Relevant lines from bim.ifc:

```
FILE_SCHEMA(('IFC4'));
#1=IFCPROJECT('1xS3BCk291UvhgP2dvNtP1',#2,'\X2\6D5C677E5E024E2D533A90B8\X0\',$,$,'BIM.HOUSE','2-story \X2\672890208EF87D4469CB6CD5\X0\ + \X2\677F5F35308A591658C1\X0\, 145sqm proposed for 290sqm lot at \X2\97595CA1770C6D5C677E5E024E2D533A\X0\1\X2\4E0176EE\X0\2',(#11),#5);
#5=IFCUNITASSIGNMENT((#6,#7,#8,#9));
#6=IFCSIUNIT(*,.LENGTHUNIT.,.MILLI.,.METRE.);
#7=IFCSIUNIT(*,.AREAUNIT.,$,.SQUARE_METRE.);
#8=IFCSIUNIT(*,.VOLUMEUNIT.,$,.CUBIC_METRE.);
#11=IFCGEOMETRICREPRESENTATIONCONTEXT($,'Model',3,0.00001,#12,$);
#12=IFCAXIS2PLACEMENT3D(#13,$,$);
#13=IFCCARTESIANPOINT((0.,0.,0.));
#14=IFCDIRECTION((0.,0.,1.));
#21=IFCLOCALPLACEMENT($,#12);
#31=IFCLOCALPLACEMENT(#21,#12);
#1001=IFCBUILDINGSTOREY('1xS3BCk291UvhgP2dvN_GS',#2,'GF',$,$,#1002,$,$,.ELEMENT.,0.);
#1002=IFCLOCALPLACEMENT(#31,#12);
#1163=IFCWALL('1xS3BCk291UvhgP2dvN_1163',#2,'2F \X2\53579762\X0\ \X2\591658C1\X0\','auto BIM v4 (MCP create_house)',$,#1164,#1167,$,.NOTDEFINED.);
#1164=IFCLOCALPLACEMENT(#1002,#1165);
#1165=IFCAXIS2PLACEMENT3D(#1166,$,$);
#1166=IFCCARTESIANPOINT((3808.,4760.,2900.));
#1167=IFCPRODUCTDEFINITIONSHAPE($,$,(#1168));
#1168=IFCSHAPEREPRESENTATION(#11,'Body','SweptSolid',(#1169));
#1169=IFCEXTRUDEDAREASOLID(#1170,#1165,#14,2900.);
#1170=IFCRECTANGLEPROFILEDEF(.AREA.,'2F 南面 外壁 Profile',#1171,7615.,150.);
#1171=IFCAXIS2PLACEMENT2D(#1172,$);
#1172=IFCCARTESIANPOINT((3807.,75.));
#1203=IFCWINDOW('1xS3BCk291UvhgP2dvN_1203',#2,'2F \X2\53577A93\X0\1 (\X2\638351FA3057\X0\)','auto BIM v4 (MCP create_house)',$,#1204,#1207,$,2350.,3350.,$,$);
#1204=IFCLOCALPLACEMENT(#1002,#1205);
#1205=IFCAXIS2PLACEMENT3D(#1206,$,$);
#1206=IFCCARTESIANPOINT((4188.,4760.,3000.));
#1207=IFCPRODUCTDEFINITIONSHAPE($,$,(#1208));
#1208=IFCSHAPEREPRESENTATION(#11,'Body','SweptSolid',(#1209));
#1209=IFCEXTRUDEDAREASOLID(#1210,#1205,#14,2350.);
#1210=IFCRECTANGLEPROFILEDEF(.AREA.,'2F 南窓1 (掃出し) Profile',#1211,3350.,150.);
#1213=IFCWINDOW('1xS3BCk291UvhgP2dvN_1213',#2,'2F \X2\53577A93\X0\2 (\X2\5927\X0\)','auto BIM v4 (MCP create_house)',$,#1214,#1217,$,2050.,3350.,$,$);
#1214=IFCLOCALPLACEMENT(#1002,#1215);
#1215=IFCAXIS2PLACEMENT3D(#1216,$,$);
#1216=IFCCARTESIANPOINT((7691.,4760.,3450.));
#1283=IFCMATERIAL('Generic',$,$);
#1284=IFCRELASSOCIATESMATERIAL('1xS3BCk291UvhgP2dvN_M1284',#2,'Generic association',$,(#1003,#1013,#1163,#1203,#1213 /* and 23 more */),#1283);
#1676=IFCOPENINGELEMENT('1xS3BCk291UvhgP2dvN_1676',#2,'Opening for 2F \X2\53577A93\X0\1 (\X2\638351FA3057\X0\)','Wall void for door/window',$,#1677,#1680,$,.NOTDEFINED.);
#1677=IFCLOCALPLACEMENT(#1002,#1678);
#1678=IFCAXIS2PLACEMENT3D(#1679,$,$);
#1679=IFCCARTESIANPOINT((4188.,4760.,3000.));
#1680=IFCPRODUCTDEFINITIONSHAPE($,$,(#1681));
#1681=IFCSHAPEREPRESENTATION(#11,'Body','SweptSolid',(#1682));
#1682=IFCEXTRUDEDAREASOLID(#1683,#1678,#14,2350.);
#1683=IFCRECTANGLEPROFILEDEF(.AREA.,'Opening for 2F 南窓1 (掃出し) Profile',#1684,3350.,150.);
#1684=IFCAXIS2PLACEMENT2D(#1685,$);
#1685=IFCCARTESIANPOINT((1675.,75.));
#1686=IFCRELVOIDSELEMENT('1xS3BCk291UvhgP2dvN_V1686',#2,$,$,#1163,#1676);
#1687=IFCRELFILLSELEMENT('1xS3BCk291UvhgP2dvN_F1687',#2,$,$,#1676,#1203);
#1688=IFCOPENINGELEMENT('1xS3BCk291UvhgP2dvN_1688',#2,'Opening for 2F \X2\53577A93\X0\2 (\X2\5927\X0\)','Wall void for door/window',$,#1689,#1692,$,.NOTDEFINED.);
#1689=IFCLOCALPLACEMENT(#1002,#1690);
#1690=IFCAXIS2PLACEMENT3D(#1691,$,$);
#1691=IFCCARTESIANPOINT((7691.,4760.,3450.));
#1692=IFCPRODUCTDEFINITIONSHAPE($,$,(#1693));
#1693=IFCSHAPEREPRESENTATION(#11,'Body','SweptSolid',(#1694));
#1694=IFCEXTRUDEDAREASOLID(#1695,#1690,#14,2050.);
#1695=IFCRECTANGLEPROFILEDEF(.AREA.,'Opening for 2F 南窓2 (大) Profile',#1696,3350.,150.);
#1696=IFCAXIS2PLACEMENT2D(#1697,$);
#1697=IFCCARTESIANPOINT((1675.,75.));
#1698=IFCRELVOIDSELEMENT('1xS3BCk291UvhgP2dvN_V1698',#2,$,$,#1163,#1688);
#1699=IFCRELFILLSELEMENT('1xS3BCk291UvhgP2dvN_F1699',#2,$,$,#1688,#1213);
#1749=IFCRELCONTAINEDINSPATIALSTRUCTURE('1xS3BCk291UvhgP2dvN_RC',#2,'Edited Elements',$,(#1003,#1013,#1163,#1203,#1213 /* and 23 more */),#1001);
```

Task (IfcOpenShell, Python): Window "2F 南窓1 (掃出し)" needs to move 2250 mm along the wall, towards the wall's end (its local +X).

```python
import ifcopenshell
import ifcopenshell.api.geometry
import ifcopenshell.util.placement

model = ifcopenshell.open("bim.ifc")

window = model.by_guid("1xS3BCk291UvhgP2dvN_1203")
opening = window.FillsVoids[0].RelatingOpeningElement
wall = opening.VoidsElements[0].RelatingBuildingElement

wall_matrix = ifcopenshell.util.placement.get_local_placement(wall.ObjectPlacement)
shift = wall_matrix[:3, 0] * 2250.0
before = ifcopenshell.util.placement.get_local_placement(window.ObjectPlacement)[:3, 3].copy()

# The window is not placed relative to its opening, so move both.
for product in (opening, window):
    matrix = ifcopenshell.util.placement.get_local_placement(product.ObjectPlacement)
    matrix[:3, 3] += shift
    ifcopenshell.api.geometry.edit_object_placement(model, product=product, matrix=matrix, is_si=False)

after = ifcopenshell.util.placement.get_local_placement(window.ObjectPlacement)[:3, 3]
print("window moved by", (after - before).round(3) + 0.0)

model.write("bim_v2.ifc")
```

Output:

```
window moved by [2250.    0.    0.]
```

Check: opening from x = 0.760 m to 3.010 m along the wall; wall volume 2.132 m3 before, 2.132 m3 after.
